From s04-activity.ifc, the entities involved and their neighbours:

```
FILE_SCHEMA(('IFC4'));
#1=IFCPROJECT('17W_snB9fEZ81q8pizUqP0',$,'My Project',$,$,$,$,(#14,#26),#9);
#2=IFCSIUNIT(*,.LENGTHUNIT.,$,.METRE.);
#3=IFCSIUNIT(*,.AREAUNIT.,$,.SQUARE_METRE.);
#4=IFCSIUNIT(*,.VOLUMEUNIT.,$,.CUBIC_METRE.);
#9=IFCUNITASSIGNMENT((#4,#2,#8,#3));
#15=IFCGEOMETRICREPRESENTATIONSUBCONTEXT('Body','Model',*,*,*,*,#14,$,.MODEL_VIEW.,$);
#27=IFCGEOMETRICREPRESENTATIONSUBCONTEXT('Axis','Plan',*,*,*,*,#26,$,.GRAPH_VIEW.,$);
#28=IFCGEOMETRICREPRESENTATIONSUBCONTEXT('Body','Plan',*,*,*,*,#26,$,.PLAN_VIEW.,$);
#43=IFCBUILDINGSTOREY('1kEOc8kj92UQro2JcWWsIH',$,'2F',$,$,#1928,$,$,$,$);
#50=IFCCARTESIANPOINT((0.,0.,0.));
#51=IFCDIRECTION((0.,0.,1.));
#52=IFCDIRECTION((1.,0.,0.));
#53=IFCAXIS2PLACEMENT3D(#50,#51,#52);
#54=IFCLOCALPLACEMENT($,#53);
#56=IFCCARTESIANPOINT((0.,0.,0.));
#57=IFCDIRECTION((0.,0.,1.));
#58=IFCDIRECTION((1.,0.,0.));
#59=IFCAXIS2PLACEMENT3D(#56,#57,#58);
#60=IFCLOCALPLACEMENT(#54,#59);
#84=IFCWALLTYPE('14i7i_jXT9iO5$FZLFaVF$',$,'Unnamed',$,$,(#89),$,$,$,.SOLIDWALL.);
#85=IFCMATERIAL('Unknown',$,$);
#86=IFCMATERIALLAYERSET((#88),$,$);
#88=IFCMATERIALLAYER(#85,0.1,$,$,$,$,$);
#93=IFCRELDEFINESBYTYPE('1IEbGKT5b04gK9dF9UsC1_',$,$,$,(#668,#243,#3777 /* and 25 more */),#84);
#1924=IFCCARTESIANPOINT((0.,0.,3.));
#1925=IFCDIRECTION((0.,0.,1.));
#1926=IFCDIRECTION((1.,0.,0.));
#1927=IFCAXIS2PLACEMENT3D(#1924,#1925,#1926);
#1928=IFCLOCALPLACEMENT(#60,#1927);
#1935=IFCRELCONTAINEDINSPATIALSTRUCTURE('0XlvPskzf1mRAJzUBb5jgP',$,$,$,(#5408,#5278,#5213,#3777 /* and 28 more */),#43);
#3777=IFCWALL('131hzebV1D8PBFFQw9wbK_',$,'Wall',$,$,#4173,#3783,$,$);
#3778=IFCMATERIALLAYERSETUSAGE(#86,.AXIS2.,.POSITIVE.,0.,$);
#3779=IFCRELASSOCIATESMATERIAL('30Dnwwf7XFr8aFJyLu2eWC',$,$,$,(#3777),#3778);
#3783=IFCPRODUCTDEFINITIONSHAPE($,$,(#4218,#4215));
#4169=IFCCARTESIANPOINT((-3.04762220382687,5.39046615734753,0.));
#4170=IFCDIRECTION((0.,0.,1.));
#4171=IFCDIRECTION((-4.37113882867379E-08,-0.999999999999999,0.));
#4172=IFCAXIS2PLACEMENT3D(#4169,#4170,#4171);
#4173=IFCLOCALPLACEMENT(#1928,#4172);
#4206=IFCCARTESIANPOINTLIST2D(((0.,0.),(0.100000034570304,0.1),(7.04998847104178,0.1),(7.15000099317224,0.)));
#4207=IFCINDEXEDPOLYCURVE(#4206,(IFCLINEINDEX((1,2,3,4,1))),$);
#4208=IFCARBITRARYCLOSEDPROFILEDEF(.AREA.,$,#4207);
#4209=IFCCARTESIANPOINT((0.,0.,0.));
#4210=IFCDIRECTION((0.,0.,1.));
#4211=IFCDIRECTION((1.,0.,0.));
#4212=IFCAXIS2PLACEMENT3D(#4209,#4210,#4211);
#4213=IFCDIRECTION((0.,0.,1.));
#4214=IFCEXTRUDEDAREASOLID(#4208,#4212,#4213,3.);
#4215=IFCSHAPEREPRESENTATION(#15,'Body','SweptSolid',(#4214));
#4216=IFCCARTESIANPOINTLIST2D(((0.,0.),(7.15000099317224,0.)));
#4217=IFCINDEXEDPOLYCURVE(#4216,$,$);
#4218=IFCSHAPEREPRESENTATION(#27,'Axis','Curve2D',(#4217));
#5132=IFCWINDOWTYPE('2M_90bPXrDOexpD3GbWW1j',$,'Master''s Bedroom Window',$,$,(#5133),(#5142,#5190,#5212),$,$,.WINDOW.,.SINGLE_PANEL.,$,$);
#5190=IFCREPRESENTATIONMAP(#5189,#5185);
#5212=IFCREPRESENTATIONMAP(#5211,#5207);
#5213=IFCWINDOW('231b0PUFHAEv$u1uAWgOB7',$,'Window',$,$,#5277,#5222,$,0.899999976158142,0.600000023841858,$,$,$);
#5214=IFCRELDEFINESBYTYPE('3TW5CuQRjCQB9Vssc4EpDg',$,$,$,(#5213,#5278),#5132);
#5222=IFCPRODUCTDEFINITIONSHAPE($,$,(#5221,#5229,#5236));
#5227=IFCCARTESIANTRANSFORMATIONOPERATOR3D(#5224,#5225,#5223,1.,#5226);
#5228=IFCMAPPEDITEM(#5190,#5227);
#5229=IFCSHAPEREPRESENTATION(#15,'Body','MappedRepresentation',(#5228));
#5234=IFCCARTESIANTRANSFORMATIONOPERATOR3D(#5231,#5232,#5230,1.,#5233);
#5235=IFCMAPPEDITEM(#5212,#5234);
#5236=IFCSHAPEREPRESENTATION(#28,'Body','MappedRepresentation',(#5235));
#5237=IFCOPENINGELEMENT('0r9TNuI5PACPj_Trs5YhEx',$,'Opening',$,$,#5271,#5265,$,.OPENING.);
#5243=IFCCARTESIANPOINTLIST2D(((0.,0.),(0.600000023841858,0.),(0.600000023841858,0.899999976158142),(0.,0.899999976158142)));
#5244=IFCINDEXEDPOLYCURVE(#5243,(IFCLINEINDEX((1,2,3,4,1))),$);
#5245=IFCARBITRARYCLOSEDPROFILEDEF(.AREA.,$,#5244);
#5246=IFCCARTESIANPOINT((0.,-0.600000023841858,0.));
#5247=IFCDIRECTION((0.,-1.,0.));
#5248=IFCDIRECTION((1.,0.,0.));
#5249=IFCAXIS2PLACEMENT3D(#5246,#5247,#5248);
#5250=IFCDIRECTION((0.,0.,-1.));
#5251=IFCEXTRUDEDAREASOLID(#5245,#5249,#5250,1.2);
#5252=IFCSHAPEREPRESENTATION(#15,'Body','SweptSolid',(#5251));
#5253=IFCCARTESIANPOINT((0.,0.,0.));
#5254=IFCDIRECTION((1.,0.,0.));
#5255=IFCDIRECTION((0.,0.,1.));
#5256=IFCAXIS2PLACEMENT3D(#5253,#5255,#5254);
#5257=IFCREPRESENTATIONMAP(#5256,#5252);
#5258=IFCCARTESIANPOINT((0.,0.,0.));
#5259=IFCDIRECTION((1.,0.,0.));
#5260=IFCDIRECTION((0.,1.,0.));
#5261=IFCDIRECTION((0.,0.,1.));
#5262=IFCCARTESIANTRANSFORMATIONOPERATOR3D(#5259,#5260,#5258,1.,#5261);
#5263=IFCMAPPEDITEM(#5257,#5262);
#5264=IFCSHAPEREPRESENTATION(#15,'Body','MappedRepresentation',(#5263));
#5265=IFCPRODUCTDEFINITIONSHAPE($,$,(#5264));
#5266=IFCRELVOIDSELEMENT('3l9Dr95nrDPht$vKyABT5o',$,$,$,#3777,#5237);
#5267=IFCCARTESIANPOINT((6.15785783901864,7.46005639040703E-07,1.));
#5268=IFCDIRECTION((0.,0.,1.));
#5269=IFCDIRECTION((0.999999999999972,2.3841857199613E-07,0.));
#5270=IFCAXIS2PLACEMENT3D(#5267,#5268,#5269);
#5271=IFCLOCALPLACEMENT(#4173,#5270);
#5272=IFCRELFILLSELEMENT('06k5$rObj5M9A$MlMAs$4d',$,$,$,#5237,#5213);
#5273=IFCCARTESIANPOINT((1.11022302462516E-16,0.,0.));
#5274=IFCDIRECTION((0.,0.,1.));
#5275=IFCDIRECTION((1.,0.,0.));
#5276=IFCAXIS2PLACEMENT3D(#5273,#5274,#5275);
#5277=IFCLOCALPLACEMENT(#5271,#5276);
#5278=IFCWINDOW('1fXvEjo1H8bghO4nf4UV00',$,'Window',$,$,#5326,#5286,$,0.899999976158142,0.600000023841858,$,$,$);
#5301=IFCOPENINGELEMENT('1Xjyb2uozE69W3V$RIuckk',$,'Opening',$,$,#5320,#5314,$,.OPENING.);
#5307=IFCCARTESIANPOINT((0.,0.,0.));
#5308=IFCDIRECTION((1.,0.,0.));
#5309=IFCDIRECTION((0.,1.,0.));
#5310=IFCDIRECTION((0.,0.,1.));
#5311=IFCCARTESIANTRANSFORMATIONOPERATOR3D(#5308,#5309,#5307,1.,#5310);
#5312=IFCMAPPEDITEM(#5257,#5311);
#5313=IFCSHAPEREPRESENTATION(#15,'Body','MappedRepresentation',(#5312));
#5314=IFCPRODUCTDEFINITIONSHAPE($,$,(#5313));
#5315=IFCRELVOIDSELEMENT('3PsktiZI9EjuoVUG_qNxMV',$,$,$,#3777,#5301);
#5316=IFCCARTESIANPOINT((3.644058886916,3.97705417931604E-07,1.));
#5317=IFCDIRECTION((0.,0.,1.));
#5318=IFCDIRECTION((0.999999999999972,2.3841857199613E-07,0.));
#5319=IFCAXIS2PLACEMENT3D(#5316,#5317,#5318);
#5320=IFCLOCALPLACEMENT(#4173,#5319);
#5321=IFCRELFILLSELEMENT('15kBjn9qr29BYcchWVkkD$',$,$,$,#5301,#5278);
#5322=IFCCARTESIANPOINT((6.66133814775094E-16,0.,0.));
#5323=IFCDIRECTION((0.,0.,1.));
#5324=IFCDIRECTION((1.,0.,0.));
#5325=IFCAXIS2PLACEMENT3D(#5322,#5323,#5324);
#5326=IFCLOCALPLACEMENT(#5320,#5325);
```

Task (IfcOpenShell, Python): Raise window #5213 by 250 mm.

```python
import numpy as np
import ifcopenshell
import ifcopenshell.api.geometry
import ifcopenshell.util.placement
import ifcopenshell.util.unit

model = ifcopenshell.open("s04-activity.ifc")
unit_scale = ifcopenshell.util.unit.calculate_unit_scale(model)

window = model.by_guid("231b0PUFHAEv$u1uAWgOB7")
opening = window.FillsVoids[0].RelatingOpeningElement
dz = 0.25

shift = np.array([0.0, 0.0, dz])
# The window is placed relative to its opening, so it follows when the opening moves.
matrix = ifcopenshell.util.placement.get_local_placement(opening.ObjectPlacement)
matrix[:3, 3] += shift
ifcopenshell.api.geometry.edit_object_placement(
    model, product=opening, matrix=matrix, is_si=False, should_transform_children=True
)

print(f"moved by {dz * unit_scale:+.3f} m")

model.write("s04-activity-out.ifc")
```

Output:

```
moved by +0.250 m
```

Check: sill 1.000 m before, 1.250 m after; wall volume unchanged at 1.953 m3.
